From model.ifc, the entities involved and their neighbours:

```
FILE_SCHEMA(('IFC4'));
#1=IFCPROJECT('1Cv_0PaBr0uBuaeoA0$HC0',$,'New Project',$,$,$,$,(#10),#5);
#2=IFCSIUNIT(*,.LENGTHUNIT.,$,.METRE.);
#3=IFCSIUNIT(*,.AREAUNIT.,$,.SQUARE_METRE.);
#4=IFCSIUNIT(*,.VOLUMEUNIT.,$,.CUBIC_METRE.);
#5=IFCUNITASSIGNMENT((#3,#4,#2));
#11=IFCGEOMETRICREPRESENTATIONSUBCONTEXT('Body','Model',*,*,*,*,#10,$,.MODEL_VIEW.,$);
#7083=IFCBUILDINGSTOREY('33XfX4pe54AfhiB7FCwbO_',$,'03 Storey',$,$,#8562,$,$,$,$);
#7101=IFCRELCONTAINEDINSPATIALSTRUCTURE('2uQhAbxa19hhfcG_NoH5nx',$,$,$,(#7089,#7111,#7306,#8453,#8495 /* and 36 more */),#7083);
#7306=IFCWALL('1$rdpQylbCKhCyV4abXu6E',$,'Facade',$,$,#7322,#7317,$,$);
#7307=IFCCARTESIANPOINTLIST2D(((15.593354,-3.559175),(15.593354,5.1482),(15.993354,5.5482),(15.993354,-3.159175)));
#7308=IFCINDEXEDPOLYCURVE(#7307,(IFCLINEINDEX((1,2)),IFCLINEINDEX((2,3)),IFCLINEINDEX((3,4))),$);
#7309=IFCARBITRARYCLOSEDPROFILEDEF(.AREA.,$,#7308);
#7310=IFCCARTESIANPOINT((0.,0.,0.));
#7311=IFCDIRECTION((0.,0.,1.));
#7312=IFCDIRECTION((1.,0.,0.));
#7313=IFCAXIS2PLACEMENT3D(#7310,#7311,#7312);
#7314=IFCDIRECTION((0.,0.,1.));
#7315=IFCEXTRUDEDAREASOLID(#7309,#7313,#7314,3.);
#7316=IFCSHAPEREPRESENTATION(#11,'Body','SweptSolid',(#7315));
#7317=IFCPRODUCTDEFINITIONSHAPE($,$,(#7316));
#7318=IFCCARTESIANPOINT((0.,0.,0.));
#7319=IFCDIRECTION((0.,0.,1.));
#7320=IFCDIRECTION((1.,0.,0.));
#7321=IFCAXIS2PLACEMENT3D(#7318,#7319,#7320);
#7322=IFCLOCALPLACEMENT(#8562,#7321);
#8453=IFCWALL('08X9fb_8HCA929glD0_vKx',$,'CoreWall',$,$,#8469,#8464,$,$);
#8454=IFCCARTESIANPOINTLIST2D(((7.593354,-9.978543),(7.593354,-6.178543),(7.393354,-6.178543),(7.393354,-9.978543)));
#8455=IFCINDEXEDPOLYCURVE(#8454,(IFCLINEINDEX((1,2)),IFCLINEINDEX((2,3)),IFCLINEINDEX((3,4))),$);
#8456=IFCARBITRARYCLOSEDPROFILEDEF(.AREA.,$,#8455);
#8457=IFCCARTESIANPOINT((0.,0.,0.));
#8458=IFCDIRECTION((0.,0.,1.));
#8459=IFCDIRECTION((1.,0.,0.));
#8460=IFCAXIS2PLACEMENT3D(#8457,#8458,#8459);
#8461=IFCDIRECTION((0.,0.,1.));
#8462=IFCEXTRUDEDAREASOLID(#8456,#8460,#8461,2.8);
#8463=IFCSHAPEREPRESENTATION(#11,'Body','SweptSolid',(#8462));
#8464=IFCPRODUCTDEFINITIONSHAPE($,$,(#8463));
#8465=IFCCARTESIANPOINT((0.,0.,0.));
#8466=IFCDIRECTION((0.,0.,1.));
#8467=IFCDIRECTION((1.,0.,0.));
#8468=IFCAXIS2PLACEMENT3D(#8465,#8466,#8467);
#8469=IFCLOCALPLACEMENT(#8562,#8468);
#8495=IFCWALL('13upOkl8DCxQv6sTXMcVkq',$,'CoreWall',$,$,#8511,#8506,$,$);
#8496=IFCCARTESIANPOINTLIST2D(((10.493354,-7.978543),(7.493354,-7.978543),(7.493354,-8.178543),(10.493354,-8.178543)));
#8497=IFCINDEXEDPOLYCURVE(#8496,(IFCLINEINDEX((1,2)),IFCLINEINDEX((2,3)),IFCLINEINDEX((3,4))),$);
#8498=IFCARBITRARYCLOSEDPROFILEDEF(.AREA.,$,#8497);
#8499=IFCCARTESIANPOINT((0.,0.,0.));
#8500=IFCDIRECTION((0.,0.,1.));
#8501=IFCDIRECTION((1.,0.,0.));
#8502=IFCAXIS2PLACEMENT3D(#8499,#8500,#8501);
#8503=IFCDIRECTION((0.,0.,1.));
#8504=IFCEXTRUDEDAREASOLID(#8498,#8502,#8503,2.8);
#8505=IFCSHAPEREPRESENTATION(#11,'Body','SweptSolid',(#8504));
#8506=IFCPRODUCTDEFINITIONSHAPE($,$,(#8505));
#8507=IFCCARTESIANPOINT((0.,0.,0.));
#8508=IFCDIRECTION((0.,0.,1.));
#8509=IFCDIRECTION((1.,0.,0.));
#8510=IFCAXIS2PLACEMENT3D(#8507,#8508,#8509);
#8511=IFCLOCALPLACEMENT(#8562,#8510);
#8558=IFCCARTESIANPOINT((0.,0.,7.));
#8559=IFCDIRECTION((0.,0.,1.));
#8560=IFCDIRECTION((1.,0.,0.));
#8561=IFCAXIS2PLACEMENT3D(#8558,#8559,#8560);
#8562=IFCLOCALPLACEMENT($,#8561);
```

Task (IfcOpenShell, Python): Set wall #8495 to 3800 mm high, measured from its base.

```python
import ifcopenshell
import ifcopenshell.geom
import ifcopenshell.util.representation
import ifcopenshell.util.shape
import ifcopenshell.util.unit

model = ifcopenshell.open("model.ifc")
unit_scale = ifcopenshell.util.unit.calculate_unit_scale(model)
settings = ifcopenshell.geom.settings()


def volume(element):
    """Net volume in cubic metres, openings subtracted."""
    shape = ifcopenshell.geom.create_shape(settings, element)
    return ifcopenshell.util.shape.get_volume(shape.geometry)


wall = model.by_guid("13upOkl8DCxQv6sTXMcVkq")
before = volume(wall)

body = ifcopenshell.util.representation.get_representation(wall, "Model", "Body")
solid = body.Items[0]
old_height = solid.Depth
solid.Depth = 3.8 / unit_scale
after = volume(wall)

print(f"height {old_height:g} -> {solid.Depth:g}, volume {before:.3f} -> {after:.3f} m3")

model.write("model_updated.ifc")
```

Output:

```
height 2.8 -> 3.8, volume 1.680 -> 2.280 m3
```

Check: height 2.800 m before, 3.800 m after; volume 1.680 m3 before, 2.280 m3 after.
